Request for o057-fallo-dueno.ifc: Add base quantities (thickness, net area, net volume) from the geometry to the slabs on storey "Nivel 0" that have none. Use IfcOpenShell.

First a look at what the model holds.

```python
import ifcopenshell
import ifcopenshell.util.element
import ifcopenshell.util.unit

model = ifcopenshell.open("o057-fallo-dueno.ifc")
print(model.schema)
for unit_type in ("LENGTHUNIT", "AREAUNIT", "VOLUMEUNIT"):
    print(unit_type, ifcopenshell.util.unit.calculate_unit_scale(model, unit_type))
storey = next(s for s in model.by_type("IfcBuildingStorey") if s.Name == "Nivel 0")
slabs = [e for e in ifcopenshell.util.element.get_decomposition(storey) if e.is_a("IfcSlab")]
for e in sorted(slabs, key=lambda e: e.id()):
    print(e.id(), e.is_a(), e.Name, list(ifcopenshell.util.element.get_psets(e, qtos_only=True)), sep=" | ")
```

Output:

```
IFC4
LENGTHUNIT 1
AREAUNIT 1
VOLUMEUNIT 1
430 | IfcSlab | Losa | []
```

```python
import ifcopenshell
import ifcopenshell.api.pset
import ifcopenshell.geom
import ifcopenshell.util.element
import ifcopenshell.util.shape
import ifcopenshell.util.unit

model = ifcopenshell.open("o057-fallo-dueno.ifc")
unit_scale = ifcopenshell.util.unit.calculate_unit_scale(model)
area_scale = ifcopenshell.util.unit.calculate_unit_scale(model, "AREAUNIT")
volume_scale = ifcopenshell.util.unit.calculate_unit_scale(model, "VOLUMEUNIT")
settings = ifcopenshell.geom.settings()

storey = next(s for s in model.by_type("IfcBuildingStorey") if s.Name == "Nivel 0")
slabs = [e for e in ifcopenshell.util.element.get_decomposition(storey) if e.is_a("IfcSlab")]

for e in sorted(slabs, key=lambda e: e.id()):
    if ifcopenshell.util.element.get_psets(e, qtos_only=True, should_inherit=False):
        continue
    # Geometry comes back in metres, in the element's own axes.
    shape = ifcopenshell.geom.create_shape(settings, e)
    values = {
        "Width": ifcopenshell.util.shape.get_z(shape.geometry) / unit_scale,
        "NetArea": ifcopenshell.util.shape.get_footprint_area(shape.geometry) / area_scale,
        "NetVolume": ifcopenshell.util.shape.get_volume(shape.geometry) / volume_scale,
    }
    qto = ifcopenshell.api.pset.add_qto(model, product=e, name="Qto_SlabBaseQuantities")
    ifcopenshell.api.pset.edit_qto(model, qto=qto, properties=values)
    print(e.id(), {k: round(v, 3) for k, v in values.items()})

model.write("o057-fallo-dueno_updated.ifc")
```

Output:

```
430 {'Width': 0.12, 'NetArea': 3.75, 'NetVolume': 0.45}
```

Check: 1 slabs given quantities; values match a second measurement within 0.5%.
